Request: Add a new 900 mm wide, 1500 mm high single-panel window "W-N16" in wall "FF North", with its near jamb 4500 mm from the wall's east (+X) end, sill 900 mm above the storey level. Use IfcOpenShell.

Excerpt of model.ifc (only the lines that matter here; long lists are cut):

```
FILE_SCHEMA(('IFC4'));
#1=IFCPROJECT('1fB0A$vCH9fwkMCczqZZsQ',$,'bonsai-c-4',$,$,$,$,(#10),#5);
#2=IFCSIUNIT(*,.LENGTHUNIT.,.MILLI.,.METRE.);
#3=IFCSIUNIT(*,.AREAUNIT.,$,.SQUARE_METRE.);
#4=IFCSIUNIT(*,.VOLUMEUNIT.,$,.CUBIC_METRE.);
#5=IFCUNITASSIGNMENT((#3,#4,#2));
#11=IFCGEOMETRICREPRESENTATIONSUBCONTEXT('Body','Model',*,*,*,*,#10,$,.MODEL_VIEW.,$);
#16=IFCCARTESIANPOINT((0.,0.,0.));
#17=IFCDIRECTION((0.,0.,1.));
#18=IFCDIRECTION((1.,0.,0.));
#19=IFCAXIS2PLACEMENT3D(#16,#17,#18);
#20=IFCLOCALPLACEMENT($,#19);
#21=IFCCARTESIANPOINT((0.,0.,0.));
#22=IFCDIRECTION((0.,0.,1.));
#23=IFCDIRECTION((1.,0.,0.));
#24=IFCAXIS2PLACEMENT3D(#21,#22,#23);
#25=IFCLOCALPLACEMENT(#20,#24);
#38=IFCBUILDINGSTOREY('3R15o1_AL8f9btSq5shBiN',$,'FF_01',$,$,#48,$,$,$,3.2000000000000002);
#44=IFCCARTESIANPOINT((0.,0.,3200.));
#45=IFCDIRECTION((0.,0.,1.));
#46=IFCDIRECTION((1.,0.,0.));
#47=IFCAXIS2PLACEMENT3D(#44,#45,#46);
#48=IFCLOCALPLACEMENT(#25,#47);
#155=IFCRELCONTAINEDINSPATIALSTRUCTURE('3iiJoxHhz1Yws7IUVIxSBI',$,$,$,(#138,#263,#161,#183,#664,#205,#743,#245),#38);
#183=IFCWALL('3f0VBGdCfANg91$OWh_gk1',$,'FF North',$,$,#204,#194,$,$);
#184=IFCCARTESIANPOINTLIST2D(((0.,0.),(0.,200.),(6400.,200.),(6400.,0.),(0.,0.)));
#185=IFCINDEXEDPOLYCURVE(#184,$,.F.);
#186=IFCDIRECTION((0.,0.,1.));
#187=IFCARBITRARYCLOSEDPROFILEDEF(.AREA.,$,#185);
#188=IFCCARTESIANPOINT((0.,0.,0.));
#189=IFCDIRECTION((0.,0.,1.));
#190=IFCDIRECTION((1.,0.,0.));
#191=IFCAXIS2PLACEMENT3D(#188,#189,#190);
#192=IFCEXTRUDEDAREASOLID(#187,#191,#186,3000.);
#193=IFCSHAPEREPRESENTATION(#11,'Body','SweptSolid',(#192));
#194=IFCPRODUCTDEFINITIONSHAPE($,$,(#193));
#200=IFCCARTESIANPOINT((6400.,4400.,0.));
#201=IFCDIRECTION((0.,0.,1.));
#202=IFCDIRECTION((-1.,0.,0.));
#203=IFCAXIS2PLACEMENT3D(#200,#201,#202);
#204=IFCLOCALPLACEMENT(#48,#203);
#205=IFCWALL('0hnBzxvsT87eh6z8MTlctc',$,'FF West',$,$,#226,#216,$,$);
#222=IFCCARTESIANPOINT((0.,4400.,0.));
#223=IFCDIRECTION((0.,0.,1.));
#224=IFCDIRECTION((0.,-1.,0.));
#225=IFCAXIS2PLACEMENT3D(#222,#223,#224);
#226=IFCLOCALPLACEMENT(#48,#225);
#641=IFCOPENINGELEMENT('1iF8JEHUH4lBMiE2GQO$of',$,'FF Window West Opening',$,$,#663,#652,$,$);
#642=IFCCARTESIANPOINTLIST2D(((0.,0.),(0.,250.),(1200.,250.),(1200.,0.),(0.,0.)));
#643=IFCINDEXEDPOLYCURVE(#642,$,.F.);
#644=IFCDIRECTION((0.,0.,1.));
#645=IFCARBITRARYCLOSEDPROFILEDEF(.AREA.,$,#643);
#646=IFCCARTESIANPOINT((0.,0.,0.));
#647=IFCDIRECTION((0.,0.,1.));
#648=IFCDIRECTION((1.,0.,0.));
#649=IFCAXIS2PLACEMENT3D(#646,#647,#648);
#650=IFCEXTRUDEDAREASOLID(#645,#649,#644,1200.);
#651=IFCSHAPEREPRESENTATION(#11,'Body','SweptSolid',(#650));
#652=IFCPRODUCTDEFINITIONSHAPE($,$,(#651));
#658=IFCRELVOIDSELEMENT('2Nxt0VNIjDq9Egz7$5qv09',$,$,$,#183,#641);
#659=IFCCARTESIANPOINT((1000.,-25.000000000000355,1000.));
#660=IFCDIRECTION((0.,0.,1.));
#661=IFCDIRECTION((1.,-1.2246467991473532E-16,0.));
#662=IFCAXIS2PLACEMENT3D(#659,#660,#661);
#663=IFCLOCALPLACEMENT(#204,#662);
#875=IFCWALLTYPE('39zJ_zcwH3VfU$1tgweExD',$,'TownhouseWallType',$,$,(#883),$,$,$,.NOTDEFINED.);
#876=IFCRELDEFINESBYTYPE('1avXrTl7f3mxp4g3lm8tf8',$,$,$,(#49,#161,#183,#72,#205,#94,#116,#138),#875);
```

```python
import numpy as np
import ifcopenshell
import ifcopenshell.api.feature
import ifcopenshell.api.geometry
import ifcopenshell.api.root
import ifcopenshell.api.spatial
import ifcopenshell.geom
import ifcopenshell.util.element
import ifcopenshell.util.placement
import ifcopenshell.util.representation
import ifcopenshell.util.shape
import ifcopenshell.util.unit

model = ifcopenshell.open("model.ifc")
unit_scale = ifcopenshell.util.unit.calculate_unit_scale(model)
settings = ifcopenshell.geom.settings()


def volume(element):
    """Net volume in cubic metres, openings subtracted."""
    shape = ifcopenshell.geom.create_shape(settings, element)
    return ifcopenshell.util.shape.get_volume(shape.geometry)


wall = model.by_id(183)
storey = ifcopenshell.util.element.get_container(wall, ifc_class="IfcBuildingStorey")
context = ifcopenshell.util.representation.get_context(model, "Model", "Body", "MODEL_VIEW")
before = volume(wall)

width, height, from_end, sill = 0.9, 1.5, 4.5, 0.9  # metres

# The wall runs along its own X axis, and the end named is its -X end.
wall_shape = ifcopenshell.geom.create_shape(settings, wall)
x, y, z = ifcopenshell.util.shape.get_vertices(wall_shape.geometry).T
start = x.min() + from_end
face, thickness = float(y.min()), float(y.max() - y.min())
wall_matrix = ifcopenshell.util.placement.get_local_placement(wall.ObjectPlacement)
level = ifcopenshell.util.placement.get_local_placement(storey.ObjectPlacement)[2, 3]


def in_wall(x, y):
    """Placement at x, y metres in the wall's axes, at sill height."""
    matrix = wall_matrix.copy()
    matrix[:, 3] = wall_matrix @ np.array([x / unit_scale, y / unit_scale, 0.0, 1.0])
    matrix[2, 3] = level + sill / unit_scale
    return matrix


# Opening: a box that overshoots both wall faces by 50 mm.
opening = ifcopenshell.api.root.create_entity(model, ifc_class="IfcOpeningElement", predefined_type="OPENING")
box = ifcopenshell.api.geometry.add_wall_representation(
    model, context=context, length=width, height=height, thickness=thickness + 0.1
)
ifcopenshell.api.geometry.assign_representation(model, product=opening, representation=box)
ifcopenshell.api.geometry.edit_object_placement(model, product=opening, matrix=in_wall(start, face - 0.05), is_si=False)
ifcopenshell.api.feature.add_feature(model, feature=opening, element=wall)

window = ifcopenshell.api.root.create_entity(model, ifc_class="IfcWindow", name="W-N16", predefined_type="WINDOW")
window.OverallWidth, window.OverallHeight = width / unit_scale, height / unit_scale
window.PartitioningType = "SINGLE_PANEL"
body = ifcopenshell.api.geometry.add_window_representation(
    model,
    context=context,
    overall_width=window.OverallWidth,
    overall_height=window.OverallHeight,
    partition_type="SINGLE_PANEL",
)
ifcopenshell.api.geometry.assign_representation(model, product=window, representation=body)
ifcopenshell.api.spatial.assign_container(model, products=[window], relating_structure=storey)
ifcopenshell.api.feature.add_filling(model, opening=opening, element=window)

# Centre the window in the wall's thickness.
ifcopenshell.api.geometry.edit_object_placement(model, product=window, matrix=in_wall(start, face), is_si=False)
window_shape = ifcopenshell.geom.create_shape(settings, window)
depth = ifcopenshell.util.shape.get_vertices(window_shape.geometry)[:, 1]
offset = face + thickness / 2 - (depth.min() + depth.max()) / 2
ifcopenshell.api.geometry.edit_object_placement(model, product=window, matrix=in_wall(start, offset), is_si=False)

after = volume(wall)

print(f"wall volume {before:.3f} -> {after:.3f} m3")

model.write("model-out.ifc")
```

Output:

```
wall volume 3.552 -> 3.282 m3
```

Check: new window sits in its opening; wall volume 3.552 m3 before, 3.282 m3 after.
